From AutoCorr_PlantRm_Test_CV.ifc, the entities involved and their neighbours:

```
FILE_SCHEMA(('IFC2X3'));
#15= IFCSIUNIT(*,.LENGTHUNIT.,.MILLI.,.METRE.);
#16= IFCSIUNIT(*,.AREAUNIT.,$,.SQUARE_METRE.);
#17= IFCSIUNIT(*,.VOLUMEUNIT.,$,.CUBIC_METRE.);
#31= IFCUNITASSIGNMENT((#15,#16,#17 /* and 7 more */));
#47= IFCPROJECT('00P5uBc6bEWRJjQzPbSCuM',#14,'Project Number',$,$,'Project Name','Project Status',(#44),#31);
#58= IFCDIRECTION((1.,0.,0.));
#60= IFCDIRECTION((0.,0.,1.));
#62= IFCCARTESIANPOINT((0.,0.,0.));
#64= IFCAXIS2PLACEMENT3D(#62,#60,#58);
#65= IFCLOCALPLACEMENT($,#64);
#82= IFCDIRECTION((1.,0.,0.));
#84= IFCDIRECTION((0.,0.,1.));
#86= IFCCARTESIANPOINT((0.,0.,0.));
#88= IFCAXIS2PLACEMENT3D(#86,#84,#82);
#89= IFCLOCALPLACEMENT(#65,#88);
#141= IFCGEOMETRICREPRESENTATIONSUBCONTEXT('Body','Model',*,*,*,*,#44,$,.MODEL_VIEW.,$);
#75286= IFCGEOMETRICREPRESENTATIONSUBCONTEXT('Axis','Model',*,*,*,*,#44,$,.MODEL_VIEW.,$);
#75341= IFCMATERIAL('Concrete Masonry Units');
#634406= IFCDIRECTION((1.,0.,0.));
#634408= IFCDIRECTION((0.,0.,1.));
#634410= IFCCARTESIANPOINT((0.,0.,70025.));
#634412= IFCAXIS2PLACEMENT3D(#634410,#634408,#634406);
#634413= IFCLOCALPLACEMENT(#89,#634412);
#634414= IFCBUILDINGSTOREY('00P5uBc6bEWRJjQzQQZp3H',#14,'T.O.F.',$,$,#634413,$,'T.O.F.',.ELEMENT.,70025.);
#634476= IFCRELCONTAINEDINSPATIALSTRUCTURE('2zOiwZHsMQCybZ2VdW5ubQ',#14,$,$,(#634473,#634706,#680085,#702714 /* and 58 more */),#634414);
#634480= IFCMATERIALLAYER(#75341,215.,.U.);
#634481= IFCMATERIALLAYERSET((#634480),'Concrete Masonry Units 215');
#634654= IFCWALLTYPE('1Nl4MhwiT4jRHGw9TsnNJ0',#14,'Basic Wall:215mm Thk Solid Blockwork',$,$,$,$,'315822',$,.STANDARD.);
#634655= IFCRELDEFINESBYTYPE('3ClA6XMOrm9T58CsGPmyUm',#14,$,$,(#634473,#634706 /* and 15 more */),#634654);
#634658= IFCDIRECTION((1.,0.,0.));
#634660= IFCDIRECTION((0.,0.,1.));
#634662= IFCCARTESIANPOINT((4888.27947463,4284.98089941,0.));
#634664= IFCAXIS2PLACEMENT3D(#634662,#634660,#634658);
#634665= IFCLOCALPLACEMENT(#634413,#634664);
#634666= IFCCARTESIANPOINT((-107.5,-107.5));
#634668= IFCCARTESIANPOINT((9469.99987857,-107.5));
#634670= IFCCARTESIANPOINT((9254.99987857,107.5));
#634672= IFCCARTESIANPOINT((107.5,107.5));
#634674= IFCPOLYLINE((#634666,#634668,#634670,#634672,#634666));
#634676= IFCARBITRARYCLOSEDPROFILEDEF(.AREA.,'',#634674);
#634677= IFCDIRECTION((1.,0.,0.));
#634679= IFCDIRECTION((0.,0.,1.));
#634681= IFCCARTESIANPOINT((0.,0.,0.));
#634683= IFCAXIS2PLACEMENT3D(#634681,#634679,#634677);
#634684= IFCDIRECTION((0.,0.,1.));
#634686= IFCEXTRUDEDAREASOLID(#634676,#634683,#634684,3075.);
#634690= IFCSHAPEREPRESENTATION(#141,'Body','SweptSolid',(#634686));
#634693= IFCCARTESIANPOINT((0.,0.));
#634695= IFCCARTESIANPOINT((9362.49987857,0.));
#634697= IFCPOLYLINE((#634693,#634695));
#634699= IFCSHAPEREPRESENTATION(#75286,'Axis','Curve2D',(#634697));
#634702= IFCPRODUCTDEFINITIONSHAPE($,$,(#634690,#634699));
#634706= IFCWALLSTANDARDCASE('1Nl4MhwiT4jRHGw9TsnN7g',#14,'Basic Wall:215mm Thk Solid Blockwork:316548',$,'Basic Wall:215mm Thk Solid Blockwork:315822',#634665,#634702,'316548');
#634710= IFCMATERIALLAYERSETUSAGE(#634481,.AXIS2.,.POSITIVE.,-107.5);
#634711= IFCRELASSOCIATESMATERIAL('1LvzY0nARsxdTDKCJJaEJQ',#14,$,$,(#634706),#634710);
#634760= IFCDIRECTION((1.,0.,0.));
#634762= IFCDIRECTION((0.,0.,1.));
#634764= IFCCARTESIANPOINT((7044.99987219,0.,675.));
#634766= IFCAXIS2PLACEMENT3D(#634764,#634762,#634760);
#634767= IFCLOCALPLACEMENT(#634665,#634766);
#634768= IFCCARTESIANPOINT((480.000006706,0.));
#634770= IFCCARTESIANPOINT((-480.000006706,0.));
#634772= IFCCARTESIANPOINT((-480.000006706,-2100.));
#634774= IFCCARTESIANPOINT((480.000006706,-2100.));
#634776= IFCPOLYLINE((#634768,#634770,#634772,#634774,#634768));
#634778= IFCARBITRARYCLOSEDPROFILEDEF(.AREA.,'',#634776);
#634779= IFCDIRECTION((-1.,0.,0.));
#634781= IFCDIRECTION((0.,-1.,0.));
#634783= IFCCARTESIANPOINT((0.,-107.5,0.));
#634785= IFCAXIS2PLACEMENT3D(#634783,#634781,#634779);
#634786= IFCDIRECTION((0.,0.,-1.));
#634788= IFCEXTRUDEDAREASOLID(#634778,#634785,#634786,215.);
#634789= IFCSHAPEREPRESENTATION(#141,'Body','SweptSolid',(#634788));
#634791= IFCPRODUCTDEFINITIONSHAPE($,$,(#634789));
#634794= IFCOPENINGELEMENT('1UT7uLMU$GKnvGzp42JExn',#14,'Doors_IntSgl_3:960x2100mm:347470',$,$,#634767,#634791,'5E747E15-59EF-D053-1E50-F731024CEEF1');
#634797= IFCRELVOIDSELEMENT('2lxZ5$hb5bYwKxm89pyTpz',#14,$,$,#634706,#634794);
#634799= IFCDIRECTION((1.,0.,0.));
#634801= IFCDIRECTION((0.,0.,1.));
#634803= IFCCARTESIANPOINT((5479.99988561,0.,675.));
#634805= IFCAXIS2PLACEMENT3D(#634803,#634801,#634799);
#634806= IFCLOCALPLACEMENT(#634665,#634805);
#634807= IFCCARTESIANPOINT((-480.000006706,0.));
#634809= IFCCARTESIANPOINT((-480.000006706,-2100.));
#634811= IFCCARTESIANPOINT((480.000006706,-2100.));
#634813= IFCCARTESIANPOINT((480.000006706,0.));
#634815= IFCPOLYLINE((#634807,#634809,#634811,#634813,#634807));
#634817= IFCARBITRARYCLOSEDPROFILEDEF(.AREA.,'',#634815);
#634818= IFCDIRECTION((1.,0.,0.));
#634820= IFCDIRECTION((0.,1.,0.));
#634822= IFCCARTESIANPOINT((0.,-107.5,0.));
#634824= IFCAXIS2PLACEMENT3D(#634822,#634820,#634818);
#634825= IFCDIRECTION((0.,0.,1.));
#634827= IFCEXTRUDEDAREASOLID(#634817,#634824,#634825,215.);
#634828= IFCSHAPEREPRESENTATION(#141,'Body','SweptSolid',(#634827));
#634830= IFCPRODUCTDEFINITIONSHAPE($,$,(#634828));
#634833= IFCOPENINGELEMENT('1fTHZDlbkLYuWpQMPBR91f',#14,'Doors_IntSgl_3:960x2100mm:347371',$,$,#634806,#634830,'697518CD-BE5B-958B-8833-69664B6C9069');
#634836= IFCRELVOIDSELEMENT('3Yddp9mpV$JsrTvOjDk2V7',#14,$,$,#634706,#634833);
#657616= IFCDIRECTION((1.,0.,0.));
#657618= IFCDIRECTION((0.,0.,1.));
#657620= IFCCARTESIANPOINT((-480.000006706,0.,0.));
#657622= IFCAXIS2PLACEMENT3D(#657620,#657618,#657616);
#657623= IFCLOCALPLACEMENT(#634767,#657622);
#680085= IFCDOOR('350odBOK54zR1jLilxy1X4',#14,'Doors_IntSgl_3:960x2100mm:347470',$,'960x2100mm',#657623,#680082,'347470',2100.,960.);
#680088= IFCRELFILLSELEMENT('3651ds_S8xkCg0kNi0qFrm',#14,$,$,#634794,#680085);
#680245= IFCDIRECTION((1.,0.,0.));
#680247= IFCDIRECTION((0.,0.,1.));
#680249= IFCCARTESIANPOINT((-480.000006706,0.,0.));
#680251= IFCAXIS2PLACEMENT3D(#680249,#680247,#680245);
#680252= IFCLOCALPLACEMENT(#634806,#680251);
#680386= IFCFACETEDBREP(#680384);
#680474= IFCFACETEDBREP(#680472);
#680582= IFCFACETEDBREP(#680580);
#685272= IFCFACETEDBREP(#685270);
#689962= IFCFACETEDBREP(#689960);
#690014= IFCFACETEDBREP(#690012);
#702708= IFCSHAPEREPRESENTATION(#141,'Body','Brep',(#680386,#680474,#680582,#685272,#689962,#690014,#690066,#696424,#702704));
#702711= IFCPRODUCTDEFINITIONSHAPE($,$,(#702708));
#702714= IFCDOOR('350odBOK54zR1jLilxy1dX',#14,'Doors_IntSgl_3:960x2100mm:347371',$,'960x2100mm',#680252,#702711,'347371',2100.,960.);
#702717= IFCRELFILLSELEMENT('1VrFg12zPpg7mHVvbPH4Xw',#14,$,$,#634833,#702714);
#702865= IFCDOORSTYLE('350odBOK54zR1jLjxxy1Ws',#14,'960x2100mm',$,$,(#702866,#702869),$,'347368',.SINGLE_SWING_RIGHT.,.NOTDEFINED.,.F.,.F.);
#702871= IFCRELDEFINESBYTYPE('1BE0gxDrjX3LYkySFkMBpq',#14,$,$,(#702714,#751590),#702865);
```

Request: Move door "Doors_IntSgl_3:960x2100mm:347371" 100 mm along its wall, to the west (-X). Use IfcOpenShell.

```python
import ifcopenshell
import ifcopenshell.api.geometry
import ifcopenshell.util.placement

model = ifcopenshell.open("AutoCorr_PlantRm_Test_CV.ifc")

door = model.by_id(702714)
opening = door.FillsVoids[0].RelatingOpeningElement
wall = opening.VoidsElements[0].RelatingBuildingElement

wall_matrix = ifcopenshell.util.placement.get_local_placement(wall.ObjectPlacement)
shift = wall_matrix[:3, 0] * -100.0
before = ifcopenshell.util.placement.get_local_placement(door.ObjectPlacement)[:3, 3].copy()

# The door is placed relative to its opening, so it follows when the opening moves.
matrix = ifcopenshell.util.placement.get_local_placement(opening.ObjectPlacement)
matrix[:3, 3] += shift
ifcopenshell.api.geometry.edit_object_placement(
    model, product=opening, matrix=matrix, is_si=False, should_transform_children=True
)

after = ifcopenshell.util.placement.get_local_placement(door.ObjectPlacement)[:3, 3]
print("door moved by", (after - before).round(3) + 0.0)

model.write("AutoCorr_PlantRm_Test_CV_v2.ifc")
```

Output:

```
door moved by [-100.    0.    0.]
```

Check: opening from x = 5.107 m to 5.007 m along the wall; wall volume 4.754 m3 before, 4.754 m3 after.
